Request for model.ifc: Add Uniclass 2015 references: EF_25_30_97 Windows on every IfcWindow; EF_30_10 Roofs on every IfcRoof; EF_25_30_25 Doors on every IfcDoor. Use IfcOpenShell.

First a look at what the model holds.

```python
import ifcopenshell

model = ifcopenshell.open("model.ifc")
print(model.schema)
print("classifications:", [c.Name for c in model.by_type("IfcClassification")])
for ifc_class in ("IfcDoor", "IfcRoof", "IfcStair", "IfcWall", "IfcWindow"):
    print(ifc_class, len(model.by_type(ifc_class)))
```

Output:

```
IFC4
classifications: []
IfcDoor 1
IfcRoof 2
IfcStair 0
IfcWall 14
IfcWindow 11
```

```python
import ifcopenshell
import ifcopenshell.api.classification

model = ifcopenshell.open("model.ifc")

system = ifcopenshell.api.classification.add_classification(model, classification="Uniclass 2015")

codes = {
    "IfcWindow": ("EF_25_30_97", "Windows"),
    "IfcRoof": ("EF_30_10", "Roofs"),
    "IfcDoor": ("EF_25_30_25", "Doors"),
}
for ifc_class, (code, name) in codes.items():
    products = model.by_type(ifc_class)
    ifcopenshell.api.classification.add_reference(
        model, products=products, classification=system, identification=code, name=name
    )
    print(code, len(products))

model.write("model_edited.ifc")
```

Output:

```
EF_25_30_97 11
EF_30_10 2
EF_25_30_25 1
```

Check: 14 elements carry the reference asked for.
